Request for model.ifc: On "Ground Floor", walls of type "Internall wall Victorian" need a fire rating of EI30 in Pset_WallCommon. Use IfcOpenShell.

First a look at what the model holds.

```python
import ifcopenshell
import ifcopenshell.util.element

model = ifcopenshell.open("model.ifc")
print(model.schema)
storey = next(s for s in model.by_type("IfcBuildingStorey") if s.Name == "Ground Floor")
walls = [e for e in ifcopenshell.util.element.get_decomposition(storey) if e.is_a("IfcWall")]
seen = {}
for e in walls:
    element_type = ifcopenshell.util.element.get_type(e)
    key = (element_type.Name if element_type != e and element_type else None, ifcopenshell.util.element.get_pset(e, "Pset_WallCommon", "FireRating"))
    seen[key] = seen.get(key, 0) + 1
for (name, value), count in sorted(seen.items(), key=str):
    print(count, "x", name, "|", value)
```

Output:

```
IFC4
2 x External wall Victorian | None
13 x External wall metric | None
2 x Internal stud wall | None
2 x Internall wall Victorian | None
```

```python
import ifcopenshell
import ifcopenshell.api.pset
import ifcopenshell.util.element

model = ifcopenshell.open("model.ifc")

storey = next(s for s in model.by_type("IfcBuildingStorey") if s.Name == "Ground Floor")
walls = [e for e in ifcopenshell.util.element.get_decomposition(storey) if e.is_a("IfcWall")]

count = 0
for e in walls:
    element_type = ifcopenshell.util.element.get_type(e)
    if element_type in (None, e) or element_type.Name != "Internall wall Victorian":
        continue
    # add_pset returns the element's existing set when there is one.
    pset = ifcopenshell.api.pset.add_pset(model, product=e, name="Pset_WallCommon")
    ifcopenshell.api.pset.edit_pset(model, pset=pset, properties={"FireRating": "EI30"})
    count += 1

print(count, "walls updated")

model.write("model-out.ifc")
```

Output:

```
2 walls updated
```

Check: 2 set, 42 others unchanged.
